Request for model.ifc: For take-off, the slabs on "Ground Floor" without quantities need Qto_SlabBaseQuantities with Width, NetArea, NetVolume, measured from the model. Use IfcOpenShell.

First a look at what the model holds.

```python
import ifcopenshell
import ifcopenshell.util.element
import ifcopenshell.util.unit

model = ifcopenshell.open("model.ifc")
print(model.schema)
for unit_type in ("LENGTHUNIT", "AREAUNIT", "VOLUMEUNIT"):
    print(unit_type, ifcopenshell.util.unit.calculate_unit_scale(model, unit_type))
storey = next(s for s in model.by_type("IfcBuildingStorey") if s.Name == "Ground Floor")
slabs = [e for e in ifcopenshell.util.element.get_decomposition(storey) if e.is_a("IfcSlab")]
for e in sorted(slabs, key=lambda e: e.id()):
    print(e.id(), e.is_a(), e.Name, list(ifcopenshell.util.element.get_psets(e, qtos_only=True)), sep=" | ")
```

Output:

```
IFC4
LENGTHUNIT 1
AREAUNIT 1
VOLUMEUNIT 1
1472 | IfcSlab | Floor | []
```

```python
import ifcopenshell
import ifcopenshell.api.pset
import ifcopenshell.geom
import ifcopenshell.util.element
import ifcopenshell.util.shape
import ifcopenshell.util.unit

model = ifcopenshell.open("model.ifc")
unit_scale = ifcopenshell.util.unit.calculate_unit_scale(model)
area_scale = ifcopenshell.util.unit.calculate_unit_scale(model, "AREAUNIT")
volume_scale = ifcopenshell.util.unit.calculate_unit_scale(model, "VOLUMEUNIT")
settings = ifcopenshell.geom.settings()

storey = next(s for s in model.by_type("IfcBuildingStorey") if s.Name == "Ground Floor")
slabs = [e for e in ifcopenshell.util.element.get_decomposition(storey) if e.is_a("IfcSlab")]

for e in sorted(slabs, key=lambda e: e.id()):
    if ifcopenshell.util.element.get_psets(e, qtos_only=True, should_inherit=False):
        continue
    # Geometry comes back in metres, in the element's own axes.
    shape = ifcopenshell.geom.create_shape(settings, e)
    values = {
        "Width": ifcopenshell.util.shape.get_z(shape.geometry) / unit_scale,
        "NetArea": ifcopenshell.util.shape.get_footprint_area(shape.geometry) / area_scale,
        "NetVolume": ifcopenshell.util.shape.get_volume(shape.geometry) / volume_scale,
    }
    qto = ifcopenshell.api.pset.add_qto(model, product=e, name="Qto_SlabBaseQuantities")
    ifcopenshell.api.pset.edit_qto(model, qto=qto, properties=values)
    print(e.id(), {k: round(v, 3) for k, v in values.items()})

model.write("model-out.ifc")
```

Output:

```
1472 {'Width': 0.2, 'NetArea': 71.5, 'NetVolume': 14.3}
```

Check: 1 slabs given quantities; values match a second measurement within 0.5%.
